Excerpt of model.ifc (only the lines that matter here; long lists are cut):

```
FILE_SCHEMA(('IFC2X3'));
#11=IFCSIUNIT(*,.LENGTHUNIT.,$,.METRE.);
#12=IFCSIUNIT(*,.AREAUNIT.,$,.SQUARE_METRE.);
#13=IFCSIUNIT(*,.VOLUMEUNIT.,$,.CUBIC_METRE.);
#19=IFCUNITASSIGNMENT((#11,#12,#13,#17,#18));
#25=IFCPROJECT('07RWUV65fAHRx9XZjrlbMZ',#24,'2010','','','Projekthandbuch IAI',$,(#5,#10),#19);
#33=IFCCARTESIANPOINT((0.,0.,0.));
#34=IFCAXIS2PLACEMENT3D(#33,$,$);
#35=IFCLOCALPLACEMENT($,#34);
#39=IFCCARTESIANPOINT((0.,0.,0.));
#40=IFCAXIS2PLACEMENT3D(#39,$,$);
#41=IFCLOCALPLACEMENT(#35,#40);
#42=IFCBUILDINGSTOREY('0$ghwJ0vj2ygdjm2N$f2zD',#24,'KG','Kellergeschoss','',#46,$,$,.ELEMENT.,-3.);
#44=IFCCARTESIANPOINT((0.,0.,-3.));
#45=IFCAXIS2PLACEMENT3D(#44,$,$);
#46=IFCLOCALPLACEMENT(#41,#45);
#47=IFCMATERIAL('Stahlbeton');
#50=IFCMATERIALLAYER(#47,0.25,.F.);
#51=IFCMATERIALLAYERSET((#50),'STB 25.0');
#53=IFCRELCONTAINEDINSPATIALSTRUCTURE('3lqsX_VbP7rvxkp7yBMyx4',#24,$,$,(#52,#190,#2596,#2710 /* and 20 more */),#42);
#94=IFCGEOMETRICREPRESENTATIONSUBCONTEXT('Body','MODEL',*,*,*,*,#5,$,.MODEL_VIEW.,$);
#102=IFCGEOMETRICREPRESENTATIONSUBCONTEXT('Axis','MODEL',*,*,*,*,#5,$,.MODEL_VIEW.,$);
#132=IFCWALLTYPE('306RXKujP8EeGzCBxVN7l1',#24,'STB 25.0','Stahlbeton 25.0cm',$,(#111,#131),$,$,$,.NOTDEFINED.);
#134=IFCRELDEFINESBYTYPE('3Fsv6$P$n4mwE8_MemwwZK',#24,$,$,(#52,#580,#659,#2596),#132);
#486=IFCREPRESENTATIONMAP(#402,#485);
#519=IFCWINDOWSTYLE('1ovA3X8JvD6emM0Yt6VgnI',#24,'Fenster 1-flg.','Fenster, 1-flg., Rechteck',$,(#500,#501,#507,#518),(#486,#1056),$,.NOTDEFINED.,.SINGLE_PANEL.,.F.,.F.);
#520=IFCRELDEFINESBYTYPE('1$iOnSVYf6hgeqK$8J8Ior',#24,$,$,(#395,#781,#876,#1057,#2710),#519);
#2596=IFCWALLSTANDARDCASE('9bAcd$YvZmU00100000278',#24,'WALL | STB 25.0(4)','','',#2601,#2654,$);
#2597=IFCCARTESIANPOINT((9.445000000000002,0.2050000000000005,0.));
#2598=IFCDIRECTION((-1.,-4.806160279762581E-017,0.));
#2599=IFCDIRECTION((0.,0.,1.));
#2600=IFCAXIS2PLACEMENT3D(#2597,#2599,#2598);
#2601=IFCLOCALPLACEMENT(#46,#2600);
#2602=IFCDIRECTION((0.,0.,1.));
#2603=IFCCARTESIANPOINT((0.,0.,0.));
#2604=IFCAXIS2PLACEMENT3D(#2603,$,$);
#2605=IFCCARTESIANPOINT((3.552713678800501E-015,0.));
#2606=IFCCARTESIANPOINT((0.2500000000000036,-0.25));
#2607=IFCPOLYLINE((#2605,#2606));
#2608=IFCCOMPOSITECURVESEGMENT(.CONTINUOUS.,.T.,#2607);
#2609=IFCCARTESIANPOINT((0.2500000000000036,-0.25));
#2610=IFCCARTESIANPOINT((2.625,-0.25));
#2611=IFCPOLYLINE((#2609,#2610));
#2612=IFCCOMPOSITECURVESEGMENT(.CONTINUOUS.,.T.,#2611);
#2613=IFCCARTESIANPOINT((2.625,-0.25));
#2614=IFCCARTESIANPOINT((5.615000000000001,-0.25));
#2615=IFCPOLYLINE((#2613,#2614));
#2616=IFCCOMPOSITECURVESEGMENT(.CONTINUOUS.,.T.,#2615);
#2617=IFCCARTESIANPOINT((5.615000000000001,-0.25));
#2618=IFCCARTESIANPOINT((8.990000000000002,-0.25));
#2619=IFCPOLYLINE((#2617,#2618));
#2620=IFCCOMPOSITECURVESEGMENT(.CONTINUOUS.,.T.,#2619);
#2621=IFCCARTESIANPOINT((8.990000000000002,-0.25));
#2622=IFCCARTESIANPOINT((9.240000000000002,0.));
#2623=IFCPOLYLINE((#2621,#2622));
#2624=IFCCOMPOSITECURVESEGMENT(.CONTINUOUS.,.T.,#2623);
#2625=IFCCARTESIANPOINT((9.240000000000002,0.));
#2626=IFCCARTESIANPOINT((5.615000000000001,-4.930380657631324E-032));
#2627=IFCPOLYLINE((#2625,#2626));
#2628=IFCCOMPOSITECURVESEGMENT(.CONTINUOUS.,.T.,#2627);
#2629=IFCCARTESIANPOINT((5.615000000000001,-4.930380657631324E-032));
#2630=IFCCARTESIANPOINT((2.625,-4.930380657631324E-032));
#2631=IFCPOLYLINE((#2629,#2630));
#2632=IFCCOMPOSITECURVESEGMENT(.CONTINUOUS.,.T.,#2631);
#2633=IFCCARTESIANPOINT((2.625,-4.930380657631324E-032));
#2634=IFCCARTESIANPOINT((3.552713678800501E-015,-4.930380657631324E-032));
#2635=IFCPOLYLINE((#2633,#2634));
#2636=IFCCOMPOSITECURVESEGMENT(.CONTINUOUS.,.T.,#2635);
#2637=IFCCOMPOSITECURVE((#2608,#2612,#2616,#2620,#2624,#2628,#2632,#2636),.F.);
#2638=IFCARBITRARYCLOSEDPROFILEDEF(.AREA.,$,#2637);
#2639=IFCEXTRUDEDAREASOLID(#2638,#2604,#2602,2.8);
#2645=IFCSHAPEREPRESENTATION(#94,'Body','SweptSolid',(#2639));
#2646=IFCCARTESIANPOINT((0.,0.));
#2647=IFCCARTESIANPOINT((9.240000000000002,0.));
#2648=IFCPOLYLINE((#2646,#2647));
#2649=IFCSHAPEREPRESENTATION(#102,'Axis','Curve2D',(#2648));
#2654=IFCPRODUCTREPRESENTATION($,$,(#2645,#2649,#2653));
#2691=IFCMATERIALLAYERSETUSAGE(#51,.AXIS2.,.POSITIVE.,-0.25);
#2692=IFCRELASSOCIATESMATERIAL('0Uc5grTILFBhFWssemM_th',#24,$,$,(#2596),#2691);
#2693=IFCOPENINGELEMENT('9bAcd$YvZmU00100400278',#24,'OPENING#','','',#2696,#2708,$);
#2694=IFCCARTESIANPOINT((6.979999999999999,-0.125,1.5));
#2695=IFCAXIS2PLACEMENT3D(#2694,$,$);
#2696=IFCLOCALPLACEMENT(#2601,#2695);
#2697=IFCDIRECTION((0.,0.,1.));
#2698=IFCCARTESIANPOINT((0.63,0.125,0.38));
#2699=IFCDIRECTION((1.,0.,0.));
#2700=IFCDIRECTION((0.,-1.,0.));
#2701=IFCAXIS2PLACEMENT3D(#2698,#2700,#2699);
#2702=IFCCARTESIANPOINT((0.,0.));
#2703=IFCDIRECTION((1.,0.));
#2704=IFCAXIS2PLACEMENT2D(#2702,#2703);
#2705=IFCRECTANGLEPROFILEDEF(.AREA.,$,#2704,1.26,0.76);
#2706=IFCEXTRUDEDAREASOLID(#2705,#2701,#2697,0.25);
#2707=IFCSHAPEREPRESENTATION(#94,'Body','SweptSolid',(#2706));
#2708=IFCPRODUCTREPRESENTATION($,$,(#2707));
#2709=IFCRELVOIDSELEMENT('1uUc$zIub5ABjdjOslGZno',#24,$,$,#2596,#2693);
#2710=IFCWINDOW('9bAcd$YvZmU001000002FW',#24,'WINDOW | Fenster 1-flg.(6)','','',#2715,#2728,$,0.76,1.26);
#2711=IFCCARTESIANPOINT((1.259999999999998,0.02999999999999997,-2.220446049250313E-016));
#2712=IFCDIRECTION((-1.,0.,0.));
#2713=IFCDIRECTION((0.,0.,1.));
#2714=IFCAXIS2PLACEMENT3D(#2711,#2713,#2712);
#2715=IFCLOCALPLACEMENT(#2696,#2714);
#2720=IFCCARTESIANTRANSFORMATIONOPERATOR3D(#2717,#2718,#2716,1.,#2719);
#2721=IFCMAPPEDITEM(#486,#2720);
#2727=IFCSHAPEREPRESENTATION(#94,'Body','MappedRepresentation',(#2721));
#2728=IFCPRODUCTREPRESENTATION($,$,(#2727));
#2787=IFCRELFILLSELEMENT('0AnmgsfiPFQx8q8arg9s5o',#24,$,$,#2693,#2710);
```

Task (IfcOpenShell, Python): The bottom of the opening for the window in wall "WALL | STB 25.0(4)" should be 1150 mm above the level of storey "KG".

```python
import numpy as np
import ifcopenshell
import ifcopenshell.api.geometry
import ifcopenshell.geom
import ifcopenshell.util.element
import ifcopenshell.util.placement
import ifcopenshell.util.shape
import ifcopenshell.util.unit

model = ifcopenshell.open("model.ifc")
unit_scale = ifcopenshell.util.unit.calculate_unit_scale(model)

window = model.by_guid("9bAcd$YvZmU001000002FW")
opening = window.FillsVoids[0].RelatingOpeningElement
storey = ifcopenshell.util.element.get_container(window, ifc_class="IfcBuildingStorey")
level = ifcopenshell.util.placement.get_local_placement(storey.ObjectPlacement)[2, 3]

# The opening's origin need not be at the sill, so measure its lowest point.
shape = ifcopenshell.geom.create_shape(ifcopenshell.geom.settings(), opening)
bottom = ifcopenshell.util.shape.get_shape_bottom_elevation(shape, shape.geometry) / unit_scale
dz = level + 1.15 - bottom

shift = np.array([0.0, 0.0, dz])
# The window is placed relative to its opening, so it follows when the opening moves.
matrix = ifcopenshell.util.placement.get_local_placement(opening.ObjectPlacement)
matrix[:3, 3] += shift
ifcopenshell.api.geometry.edit_object_placement(
    model, product=opening, matrix=matrix, is_si=False, should_transform_children=True
)

print(f"moved by {dz * unit_scale:+.3f} m")

model.write("model_edited.ifc")
```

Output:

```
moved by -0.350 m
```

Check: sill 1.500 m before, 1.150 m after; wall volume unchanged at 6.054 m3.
